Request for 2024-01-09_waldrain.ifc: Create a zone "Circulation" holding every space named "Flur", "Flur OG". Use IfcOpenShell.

First a look at what the model holds.

```python
import ifcopenshell

model = ifcopenshell.open("2024-01-09_waldrain.ifc")
print(model.schema)
seen = {}
for space in model.by_type("IfcSpace"):
    seen[space.LongName] = seen.get(space.LongName, 0) + 1
for name, count in sorted(seen.items(), key=str):
    print(count, "x", name)
print("zones:", [z.Name for z in model.by_type("IfcZone")][:20])
```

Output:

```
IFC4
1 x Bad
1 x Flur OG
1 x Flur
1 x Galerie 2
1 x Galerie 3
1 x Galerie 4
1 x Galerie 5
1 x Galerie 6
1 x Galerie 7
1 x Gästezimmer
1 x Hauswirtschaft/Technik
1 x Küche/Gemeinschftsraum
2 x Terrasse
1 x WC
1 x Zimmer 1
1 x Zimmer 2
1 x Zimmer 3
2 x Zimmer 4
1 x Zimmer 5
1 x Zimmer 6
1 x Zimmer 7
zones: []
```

```python
import ifcopenshell
import ifcopenshell.api.group
import ifcopenshell.api.root

model = ifcopenshell.open("2024-01-09_waldrain.ifc")

names = {"Flur", "Flur OG"}
spaces = [s for s in model.by_type("IfcSpace") if s.LongName in names]

zone = ifcopenshell.api.root.create_entity(model, ifc_class="IfcZone", name="Circulation")
ifcopenshell.api.group.assign_group(model, products=spaces, group=zone)
print(len(spaces), "spaces in", zone.Name)

model.write("2024-01-09_waldrain_rev.ifc")
```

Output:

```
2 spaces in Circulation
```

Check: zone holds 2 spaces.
